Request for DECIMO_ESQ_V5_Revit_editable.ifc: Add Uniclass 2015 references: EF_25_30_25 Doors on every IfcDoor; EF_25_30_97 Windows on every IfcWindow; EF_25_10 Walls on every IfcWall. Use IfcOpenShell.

First a look at what the model holds.

```python
import ifcopenshell

model = ifcopenshell.open("DECIMO_ESQ_V5_Revit_editable.ifc")
print(model.schema)
print("classifications:", [c.Name for c in model.by_type("IfcClassification")])
for ifc_class in ("IfcDoor", "IfcRoof", "IfcStair", "IfcWall", "IfcWindow"):
    print(ifc_class, len(model.by_type(ifc_class)))
```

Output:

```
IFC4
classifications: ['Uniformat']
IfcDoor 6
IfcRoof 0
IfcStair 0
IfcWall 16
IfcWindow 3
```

```python
import ifcopenshell
import ifcopenshell.api.classification

model = ifcopenshell.open("DECIMO_ESQ_V5_Revit_editable.ifc")

system = ifcopenshell.api.classification.add_classification(model, classification="Uniclass 2015")

codes = {
    "IfcDoor": ("EF_25_30_25", "Doors"),
    "IfcWindow": ("EF_25_30_97", "Windows"),
    "IfcWall": ("EF_25_10", "Walls"),
}
for ifc_class, (code, name) in codes.items():
    products = model.by_type(ifc_class)
    ifcopenshell.api.classification.add_reference(
        model, products=products, classification=system, identification=code, name=name
    )
    print(code, len(products))

model.write("DECIMO_ESQ_V5_Revit_editable_edited.ifc")
```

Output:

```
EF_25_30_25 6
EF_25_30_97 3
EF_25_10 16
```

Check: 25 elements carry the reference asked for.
